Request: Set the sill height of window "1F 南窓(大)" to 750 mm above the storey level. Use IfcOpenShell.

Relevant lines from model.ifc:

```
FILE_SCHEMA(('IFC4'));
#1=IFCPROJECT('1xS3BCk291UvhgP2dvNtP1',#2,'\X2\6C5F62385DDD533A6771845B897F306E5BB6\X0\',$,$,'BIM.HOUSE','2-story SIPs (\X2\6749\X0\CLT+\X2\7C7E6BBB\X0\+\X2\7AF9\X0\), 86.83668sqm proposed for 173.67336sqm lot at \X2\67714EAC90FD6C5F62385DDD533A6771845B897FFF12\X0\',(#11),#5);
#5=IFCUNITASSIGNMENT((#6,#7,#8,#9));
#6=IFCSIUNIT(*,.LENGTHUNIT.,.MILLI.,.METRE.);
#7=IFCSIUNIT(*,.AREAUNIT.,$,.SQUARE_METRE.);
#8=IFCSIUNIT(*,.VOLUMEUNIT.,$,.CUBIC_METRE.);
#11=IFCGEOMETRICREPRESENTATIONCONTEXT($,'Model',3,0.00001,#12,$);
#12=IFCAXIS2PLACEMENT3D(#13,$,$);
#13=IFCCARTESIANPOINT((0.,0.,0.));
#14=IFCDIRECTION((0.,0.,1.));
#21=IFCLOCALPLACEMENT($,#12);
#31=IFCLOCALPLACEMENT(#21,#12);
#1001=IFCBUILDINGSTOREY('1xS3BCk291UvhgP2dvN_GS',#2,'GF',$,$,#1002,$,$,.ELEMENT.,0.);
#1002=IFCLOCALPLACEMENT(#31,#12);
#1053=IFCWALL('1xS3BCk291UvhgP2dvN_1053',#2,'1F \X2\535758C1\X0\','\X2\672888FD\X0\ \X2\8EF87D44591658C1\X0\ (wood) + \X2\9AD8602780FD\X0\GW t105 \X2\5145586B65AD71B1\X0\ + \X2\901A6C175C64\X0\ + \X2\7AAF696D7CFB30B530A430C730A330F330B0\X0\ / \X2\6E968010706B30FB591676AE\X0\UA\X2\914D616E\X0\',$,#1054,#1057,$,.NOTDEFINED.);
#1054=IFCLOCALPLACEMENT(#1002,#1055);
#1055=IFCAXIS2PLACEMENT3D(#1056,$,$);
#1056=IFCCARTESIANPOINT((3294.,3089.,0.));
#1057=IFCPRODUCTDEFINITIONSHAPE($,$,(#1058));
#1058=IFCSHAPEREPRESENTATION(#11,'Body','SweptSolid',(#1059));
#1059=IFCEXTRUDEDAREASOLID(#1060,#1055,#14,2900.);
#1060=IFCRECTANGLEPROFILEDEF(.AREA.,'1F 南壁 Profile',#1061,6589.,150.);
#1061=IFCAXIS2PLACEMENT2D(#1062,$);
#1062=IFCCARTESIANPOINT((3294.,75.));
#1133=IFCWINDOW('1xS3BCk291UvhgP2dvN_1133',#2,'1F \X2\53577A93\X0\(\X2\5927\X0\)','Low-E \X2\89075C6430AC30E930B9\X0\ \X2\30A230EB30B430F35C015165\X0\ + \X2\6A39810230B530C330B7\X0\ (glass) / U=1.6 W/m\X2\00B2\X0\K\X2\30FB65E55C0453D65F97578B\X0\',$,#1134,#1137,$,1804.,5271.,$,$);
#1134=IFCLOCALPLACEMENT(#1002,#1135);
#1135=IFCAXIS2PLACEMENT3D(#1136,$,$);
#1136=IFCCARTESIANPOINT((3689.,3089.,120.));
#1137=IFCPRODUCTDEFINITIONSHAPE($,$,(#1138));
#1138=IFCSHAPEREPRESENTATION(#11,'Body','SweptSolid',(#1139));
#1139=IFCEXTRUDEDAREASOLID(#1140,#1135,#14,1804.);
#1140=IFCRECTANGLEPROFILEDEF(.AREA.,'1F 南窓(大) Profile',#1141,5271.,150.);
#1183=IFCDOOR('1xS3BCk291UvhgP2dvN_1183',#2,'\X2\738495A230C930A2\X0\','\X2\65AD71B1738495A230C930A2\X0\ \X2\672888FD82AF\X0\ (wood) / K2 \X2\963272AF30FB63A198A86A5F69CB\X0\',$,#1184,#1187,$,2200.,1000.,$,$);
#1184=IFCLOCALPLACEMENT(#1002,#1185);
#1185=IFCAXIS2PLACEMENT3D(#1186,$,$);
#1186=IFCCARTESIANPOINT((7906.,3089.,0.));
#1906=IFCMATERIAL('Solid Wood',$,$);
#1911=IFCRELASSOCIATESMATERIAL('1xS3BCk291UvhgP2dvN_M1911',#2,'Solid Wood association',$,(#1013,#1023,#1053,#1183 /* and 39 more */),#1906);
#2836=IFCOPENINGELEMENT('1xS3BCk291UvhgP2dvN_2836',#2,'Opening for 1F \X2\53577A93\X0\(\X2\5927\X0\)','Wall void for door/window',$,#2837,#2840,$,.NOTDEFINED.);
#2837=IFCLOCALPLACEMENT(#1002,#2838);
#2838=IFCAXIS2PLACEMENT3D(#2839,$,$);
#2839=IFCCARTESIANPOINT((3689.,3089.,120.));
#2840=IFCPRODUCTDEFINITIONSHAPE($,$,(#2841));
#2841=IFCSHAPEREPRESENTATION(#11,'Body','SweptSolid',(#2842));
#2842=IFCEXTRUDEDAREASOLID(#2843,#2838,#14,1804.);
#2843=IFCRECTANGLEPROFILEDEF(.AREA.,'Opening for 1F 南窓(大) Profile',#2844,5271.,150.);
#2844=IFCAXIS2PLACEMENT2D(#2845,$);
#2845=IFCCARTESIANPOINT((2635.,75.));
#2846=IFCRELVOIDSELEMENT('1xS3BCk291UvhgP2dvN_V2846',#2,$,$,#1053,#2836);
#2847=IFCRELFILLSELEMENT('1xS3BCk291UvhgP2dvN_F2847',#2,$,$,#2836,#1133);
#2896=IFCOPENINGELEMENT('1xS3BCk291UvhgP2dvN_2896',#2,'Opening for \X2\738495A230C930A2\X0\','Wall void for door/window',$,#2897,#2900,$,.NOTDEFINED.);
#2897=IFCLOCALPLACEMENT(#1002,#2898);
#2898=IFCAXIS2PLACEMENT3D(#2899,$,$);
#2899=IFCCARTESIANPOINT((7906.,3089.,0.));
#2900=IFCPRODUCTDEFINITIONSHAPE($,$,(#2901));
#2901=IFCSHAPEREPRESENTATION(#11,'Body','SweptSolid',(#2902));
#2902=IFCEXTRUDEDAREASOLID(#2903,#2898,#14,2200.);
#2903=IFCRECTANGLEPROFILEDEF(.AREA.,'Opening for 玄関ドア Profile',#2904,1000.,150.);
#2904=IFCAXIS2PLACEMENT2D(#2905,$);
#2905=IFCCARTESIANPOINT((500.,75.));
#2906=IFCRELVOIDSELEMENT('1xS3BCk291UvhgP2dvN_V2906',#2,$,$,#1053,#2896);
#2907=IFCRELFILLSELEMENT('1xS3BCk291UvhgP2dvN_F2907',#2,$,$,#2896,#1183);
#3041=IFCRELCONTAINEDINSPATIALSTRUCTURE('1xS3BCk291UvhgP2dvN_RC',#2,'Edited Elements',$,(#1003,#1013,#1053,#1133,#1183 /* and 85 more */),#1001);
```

```python
import numpy as np
import ifcopenshell
import ifcopenshell.api.geometry
import ifcopenshell.geom
import ifcopenshell.util.element
import ifcopenshell.util.placement
import ifcopenshell.util.shape
import ifcopenshell.util.unit

model = ifcopenshell.open("model.ifc")
unit_scale = ifcopenshell.util.unit.calculate_unit_scale(model)

window = model.by_guid("1xS3BCk291UvhgP2dvN_1133")
opening = window.FillsVoids[0].RelatingOpeningElement
storey = ifcopenshell.util.element.get_container(window, ifc_class="IfcBuildingStorey")
level = ifcopenshell.util.placement.get_local_placement(storey.ObjectPlacement)[2, 3]

# The opening's origin need not be at the sill, so measure its lowest point.
shape = ifcopenshell.geom.create_shape(ifcopenshell.geom.settings(), opening)
bottom = ifcopenshell.util.shape.get_shape_bottom_elevation(shape, shape.geometry) / unit_scale
dz = level + 0.75 / unit_scale - bottom

shift = np.array([0.0, 0.0, dz])
# The window is not placed relative to its opening, so move both.
for product in (opening, window):
    matrix = ifcopenshell.util.placement.get_local_placement(product.ObjectPlacement)
    matrix[:3, 3] += shift
    ifcopenshell.api.geometry.edit_object_placement(model, product=product, matrix=matrix, is_si=False)

print(f"moved by {dz * unit_scale:+.3f} m")

model.write("model_rev.ifc")
```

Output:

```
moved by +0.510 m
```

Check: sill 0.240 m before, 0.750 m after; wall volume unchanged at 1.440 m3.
